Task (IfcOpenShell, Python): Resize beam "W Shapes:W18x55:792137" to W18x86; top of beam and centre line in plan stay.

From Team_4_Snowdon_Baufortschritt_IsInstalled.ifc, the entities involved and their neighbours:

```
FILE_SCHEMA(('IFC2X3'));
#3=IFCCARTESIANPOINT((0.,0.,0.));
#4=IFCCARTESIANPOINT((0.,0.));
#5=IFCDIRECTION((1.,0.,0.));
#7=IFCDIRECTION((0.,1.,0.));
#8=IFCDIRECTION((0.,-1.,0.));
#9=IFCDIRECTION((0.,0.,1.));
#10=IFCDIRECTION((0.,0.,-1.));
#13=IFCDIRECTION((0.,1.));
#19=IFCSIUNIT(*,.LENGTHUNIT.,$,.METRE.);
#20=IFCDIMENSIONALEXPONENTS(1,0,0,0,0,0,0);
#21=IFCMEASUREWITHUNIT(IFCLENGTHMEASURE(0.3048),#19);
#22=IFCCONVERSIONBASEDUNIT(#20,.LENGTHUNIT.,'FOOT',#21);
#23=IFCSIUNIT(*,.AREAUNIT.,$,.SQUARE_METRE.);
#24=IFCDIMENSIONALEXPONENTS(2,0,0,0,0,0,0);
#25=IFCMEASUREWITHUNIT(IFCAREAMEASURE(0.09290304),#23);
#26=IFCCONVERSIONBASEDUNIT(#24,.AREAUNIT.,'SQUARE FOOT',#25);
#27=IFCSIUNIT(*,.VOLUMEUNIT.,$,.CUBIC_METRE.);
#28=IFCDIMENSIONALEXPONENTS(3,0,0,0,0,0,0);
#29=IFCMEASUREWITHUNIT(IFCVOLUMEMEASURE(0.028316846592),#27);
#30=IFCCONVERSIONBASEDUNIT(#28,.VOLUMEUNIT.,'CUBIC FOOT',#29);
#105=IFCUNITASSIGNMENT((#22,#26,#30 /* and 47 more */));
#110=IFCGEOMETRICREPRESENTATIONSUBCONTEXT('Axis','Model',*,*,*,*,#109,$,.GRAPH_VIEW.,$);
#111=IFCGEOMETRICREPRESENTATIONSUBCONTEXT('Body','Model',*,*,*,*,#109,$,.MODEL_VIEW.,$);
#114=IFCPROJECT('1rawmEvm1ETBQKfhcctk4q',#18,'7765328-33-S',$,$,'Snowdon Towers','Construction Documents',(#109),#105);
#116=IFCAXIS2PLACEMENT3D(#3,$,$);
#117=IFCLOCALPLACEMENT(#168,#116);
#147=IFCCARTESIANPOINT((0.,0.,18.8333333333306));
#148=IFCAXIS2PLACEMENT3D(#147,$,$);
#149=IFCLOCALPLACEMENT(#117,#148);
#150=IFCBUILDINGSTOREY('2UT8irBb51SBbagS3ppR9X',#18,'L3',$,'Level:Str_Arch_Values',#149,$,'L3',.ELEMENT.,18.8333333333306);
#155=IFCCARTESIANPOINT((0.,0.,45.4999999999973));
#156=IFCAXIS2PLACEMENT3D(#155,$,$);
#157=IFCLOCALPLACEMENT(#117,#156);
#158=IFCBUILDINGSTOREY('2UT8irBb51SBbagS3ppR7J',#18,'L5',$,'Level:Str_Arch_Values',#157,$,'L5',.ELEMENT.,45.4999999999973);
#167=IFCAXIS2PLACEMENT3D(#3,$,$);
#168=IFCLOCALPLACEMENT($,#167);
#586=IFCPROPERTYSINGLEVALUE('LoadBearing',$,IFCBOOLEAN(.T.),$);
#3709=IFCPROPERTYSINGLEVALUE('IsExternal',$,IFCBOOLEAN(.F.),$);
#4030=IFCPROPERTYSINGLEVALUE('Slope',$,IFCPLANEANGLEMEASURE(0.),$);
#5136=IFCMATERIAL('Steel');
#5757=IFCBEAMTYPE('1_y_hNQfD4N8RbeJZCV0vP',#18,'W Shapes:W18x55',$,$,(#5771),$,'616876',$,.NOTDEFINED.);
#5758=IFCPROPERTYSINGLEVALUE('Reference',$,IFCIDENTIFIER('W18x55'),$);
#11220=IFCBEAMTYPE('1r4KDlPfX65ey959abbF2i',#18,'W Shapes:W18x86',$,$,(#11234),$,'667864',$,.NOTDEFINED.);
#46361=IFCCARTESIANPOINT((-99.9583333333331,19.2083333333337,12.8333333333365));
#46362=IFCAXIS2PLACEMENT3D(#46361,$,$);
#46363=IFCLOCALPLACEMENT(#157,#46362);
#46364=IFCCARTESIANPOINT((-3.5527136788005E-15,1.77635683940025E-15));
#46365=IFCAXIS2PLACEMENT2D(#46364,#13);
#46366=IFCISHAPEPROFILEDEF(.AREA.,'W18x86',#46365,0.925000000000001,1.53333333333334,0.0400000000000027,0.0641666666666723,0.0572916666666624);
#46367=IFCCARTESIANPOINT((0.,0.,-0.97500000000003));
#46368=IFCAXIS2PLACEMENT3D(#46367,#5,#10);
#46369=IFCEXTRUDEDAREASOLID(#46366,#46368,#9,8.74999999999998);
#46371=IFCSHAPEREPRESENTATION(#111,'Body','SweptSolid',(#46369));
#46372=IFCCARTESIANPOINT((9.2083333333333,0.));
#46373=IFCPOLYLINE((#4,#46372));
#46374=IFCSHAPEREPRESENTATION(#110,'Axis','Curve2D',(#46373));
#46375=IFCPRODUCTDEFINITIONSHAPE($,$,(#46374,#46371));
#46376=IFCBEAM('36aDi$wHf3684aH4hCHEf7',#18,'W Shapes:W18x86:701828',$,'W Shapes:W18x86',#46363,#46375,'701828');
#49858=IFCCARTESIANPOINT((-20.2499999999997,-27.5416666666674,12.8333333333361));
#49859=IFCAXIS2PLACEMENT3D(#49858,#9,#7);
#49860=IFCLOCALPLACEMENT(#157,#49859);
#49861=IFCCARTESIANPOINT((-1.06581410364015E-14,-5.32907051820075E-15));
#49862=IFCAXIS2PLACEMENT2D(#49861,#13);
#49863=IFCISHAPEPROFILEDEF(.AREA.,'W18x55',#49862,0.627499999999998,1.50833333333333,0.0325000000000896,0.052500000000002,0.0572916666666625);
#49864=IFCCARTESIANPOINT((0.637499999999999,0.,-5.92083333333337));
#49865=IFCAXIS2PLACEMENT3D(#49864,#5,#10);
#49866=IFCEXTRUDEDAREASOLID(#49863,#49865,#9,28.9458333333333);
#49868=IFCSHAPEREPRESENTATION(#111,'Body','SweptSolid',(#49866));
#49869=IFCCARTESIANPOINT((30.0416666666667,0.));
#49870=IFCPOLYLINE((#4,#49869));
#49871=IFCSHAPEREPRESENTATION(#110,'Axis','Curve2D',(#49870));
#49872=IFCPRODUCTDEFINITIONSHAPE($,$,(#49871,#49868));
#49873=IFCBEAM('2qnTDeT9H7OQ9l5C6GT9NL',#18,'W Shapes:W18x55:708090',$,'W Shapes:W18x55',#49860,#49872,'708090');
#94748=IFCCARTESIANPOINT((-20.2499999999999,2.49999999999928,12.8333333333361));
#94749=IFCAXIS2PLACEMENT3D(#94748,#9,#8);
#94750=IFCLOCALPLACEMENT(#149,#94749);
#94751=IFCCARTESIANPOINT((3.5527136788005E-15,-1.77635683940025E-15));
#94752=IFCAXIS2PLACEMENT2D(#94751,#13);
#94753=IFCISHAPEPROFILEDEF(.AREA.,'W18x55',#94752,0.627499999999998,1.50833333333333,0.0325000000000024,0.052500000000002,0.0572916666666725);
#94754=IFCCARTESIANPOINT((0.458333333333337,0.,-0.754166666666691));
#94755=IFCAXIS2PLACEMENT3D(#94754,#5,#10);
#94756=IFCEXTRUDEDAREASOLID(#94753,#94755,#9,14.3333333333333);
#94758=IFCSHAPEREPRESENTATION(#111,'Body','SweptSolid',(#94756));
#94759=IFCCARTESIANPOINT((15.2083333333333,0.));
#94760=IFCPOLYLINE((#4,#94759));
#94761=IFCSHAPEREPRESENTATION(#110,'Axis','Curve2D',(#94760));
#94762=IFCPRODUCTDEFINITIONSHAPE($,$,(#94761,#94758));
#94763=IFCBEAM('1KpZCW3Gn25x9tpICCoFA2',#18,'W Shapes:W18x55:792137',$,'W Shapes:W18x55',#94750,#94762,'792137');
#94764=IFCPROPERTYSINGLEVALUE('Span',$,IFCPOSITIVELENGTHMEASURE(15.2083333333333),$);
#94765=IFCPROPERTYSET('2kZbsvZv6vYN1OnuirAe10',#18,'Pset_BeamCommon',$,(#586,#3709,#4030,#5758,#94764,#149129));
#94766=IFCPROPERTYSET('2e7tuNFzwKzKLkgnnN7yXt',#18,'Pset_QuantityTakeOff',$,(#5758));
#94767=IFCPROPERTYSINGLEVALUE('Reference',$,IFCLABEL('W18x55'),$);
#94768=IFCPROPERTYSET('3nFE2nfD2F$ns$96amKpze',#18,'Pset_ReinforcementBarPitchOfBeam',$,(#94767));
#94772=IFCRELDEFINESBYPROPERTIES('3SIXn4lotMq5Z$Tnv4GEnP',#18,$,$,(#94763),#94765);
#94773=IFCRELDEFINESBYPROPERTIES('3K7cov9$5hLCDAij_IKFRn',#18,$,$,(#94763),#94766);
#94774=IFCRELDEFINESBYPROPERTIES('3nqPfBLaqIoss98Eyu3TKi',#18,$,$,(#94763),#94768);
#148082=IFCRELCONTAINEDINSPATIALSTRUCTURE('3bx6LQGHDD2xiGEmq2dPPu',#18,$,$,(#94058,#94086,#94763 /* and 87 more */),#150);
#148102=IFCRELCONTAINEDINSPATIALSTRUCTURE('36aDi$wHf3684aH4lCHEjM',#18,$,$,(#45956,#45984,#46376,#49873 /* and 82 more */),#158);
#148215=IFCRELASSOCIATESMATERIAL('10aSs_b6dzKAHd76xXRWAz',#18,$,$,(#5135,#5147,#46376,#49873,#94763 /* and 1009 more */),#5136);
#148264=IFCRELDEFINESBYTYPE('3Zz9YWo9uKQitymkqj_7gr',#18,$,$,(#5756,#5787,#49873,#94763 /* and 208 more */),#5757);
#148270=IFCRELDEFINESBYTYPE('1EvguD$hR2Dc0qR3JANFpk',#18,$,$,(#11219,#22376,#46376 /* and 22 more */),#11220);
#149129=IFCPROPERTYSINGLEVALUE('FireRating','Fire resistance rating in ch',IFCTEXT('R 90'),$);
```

```python
import ifcopenshell
import ifcopenshell.api.pset
import ifcopenshell.api.type
import ifcopenshell.util.element
import ifcopenshell.util.representation

model = ifcopenshell.open("Team_4_Snowdon_Baufortschritt_IsInstalled.ifc")

member = model.by_guid("1KpZCW3Gn25x9tpICCoFA2")
source = next(p for p in model.by_type("IfcIShapeProfileDef") if p.ProfileName == "W18x86")

body = ifcopenshell.util.representation.get_representation(member, "Model", "Body")
solid = body.Items[0]
old_profile = solid.SweptArea

# Copy the section's sizes but keep this member's own profile position.
profile = ifcopenshell.util.element.copy(model, source)
# Profiles are centred, so shift by half the change in depth to hold the top.
shift = (old_profile.OverallDepth - profile.OverallDepth) / 2
x, y = old_profile.Position.Location.Coordinates
up = (-1.0, 0.0)  # upwards, in the solid's own plane
location = model.createIfcCartesianPoint((x + up[0] * shift, y + up[1] * shift))
profile.Position = model.createIfcAxis2Placement2D(location, old_profile.Position.RefDirection)
solid.SweptArea = profile
if not model.get_total_inverses(old_profile):
    ifcopenshell.util.element.remove_deep2(model, old_profile)

new_type = model.by_id(11220)
ifcopenshell.api.type.assign_type(
    model, related_objects=[member], relating_type=new_type, should_map_representations=False
)
member.Name = member.Name.replace("W18x55", "W18x86")
member.ObjectType = "W Shapes:W18x86"
pset = model.by_id(ifcopenshell.util.element.get_pset(member, "Pset_BeamCommon", should_inherit=False)["id"])
ifcopenshell.api.pset.edit_pset(model, pset=pset, properties={"Reference": "W18x86"})
pset = model.by_id(ifcopenshell.util.element.get_pset(member, "Pset_QuantityTakeOff", should_inherit=False)["id"])
ifcopenshell.api.pset.edit_pset(model, pset=pset, properties={"Reference": "W18x86"})
pset = model.by_id(ifcopenshell.util.element.get_pset(member, "Pset_ReinforcementBarPitchOfBeam", should_inherit=False)["id"])
ifcopenshell.api.pset.edit_pset(model, pset=pset, properties={"Reference": "W18x86"})

print(solid.SweptArea)

model.write("Team_4_Snowdon_Baufortschritt_IsInstalled_rev.ifc")
```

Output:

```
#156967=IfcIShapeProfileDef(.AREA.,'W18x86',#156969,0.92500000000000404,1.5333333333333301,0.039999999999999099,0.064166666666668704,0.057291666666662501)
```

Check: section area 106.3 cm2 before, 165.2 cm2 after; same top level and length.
